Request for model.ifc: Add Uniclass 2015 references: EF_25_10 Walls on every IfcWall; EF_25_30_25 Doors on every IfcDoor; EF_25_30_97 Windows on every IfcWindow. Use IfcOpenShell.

First a look at what the model holds.

```python
import ifcopenshell

model = ifcopenshell.open("model.ifc")
print(model.schema)
print("classifications:", [c.Name for c in model.by_type("IfcClassification")])
for ifc_class in ("IfcDoor", "IfcRoof", "IfcStair", "IfcWall", "IfcWindow"):
    print(ifc_class, len(model.by_type(ifc_class)))
```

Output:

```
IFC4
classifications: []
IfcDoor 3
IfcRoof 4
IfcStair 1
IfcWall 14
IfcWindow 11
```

```python
import ifcopenshell
import ifcopenshell.api.classification

model = ifcopenshell.open("model.ifc")

system = ifcopenshell.api.classification.add_classification(model, classification="Uniclass 2015")

codes = {
    "IfcWall": ("EF_25_10", "Walls"),
    "IfcDoor": ("EF_25_30_25", "Doors"),
    "IfcWindow": ("EF_25_30_97", "Windows"),
}
for ifc_class, (code, name) in codes.items():
    products = model.by_type(ifc_class)
    ifcopenshell.api.classification.add_reference(
        model, products=products, classification=system, identification=code, name=name
    )
    print(code, len(products))

model.write("model-out.ifc")
```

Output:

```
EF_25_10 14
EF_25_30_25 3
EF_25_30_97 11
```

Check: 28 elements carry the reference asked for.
